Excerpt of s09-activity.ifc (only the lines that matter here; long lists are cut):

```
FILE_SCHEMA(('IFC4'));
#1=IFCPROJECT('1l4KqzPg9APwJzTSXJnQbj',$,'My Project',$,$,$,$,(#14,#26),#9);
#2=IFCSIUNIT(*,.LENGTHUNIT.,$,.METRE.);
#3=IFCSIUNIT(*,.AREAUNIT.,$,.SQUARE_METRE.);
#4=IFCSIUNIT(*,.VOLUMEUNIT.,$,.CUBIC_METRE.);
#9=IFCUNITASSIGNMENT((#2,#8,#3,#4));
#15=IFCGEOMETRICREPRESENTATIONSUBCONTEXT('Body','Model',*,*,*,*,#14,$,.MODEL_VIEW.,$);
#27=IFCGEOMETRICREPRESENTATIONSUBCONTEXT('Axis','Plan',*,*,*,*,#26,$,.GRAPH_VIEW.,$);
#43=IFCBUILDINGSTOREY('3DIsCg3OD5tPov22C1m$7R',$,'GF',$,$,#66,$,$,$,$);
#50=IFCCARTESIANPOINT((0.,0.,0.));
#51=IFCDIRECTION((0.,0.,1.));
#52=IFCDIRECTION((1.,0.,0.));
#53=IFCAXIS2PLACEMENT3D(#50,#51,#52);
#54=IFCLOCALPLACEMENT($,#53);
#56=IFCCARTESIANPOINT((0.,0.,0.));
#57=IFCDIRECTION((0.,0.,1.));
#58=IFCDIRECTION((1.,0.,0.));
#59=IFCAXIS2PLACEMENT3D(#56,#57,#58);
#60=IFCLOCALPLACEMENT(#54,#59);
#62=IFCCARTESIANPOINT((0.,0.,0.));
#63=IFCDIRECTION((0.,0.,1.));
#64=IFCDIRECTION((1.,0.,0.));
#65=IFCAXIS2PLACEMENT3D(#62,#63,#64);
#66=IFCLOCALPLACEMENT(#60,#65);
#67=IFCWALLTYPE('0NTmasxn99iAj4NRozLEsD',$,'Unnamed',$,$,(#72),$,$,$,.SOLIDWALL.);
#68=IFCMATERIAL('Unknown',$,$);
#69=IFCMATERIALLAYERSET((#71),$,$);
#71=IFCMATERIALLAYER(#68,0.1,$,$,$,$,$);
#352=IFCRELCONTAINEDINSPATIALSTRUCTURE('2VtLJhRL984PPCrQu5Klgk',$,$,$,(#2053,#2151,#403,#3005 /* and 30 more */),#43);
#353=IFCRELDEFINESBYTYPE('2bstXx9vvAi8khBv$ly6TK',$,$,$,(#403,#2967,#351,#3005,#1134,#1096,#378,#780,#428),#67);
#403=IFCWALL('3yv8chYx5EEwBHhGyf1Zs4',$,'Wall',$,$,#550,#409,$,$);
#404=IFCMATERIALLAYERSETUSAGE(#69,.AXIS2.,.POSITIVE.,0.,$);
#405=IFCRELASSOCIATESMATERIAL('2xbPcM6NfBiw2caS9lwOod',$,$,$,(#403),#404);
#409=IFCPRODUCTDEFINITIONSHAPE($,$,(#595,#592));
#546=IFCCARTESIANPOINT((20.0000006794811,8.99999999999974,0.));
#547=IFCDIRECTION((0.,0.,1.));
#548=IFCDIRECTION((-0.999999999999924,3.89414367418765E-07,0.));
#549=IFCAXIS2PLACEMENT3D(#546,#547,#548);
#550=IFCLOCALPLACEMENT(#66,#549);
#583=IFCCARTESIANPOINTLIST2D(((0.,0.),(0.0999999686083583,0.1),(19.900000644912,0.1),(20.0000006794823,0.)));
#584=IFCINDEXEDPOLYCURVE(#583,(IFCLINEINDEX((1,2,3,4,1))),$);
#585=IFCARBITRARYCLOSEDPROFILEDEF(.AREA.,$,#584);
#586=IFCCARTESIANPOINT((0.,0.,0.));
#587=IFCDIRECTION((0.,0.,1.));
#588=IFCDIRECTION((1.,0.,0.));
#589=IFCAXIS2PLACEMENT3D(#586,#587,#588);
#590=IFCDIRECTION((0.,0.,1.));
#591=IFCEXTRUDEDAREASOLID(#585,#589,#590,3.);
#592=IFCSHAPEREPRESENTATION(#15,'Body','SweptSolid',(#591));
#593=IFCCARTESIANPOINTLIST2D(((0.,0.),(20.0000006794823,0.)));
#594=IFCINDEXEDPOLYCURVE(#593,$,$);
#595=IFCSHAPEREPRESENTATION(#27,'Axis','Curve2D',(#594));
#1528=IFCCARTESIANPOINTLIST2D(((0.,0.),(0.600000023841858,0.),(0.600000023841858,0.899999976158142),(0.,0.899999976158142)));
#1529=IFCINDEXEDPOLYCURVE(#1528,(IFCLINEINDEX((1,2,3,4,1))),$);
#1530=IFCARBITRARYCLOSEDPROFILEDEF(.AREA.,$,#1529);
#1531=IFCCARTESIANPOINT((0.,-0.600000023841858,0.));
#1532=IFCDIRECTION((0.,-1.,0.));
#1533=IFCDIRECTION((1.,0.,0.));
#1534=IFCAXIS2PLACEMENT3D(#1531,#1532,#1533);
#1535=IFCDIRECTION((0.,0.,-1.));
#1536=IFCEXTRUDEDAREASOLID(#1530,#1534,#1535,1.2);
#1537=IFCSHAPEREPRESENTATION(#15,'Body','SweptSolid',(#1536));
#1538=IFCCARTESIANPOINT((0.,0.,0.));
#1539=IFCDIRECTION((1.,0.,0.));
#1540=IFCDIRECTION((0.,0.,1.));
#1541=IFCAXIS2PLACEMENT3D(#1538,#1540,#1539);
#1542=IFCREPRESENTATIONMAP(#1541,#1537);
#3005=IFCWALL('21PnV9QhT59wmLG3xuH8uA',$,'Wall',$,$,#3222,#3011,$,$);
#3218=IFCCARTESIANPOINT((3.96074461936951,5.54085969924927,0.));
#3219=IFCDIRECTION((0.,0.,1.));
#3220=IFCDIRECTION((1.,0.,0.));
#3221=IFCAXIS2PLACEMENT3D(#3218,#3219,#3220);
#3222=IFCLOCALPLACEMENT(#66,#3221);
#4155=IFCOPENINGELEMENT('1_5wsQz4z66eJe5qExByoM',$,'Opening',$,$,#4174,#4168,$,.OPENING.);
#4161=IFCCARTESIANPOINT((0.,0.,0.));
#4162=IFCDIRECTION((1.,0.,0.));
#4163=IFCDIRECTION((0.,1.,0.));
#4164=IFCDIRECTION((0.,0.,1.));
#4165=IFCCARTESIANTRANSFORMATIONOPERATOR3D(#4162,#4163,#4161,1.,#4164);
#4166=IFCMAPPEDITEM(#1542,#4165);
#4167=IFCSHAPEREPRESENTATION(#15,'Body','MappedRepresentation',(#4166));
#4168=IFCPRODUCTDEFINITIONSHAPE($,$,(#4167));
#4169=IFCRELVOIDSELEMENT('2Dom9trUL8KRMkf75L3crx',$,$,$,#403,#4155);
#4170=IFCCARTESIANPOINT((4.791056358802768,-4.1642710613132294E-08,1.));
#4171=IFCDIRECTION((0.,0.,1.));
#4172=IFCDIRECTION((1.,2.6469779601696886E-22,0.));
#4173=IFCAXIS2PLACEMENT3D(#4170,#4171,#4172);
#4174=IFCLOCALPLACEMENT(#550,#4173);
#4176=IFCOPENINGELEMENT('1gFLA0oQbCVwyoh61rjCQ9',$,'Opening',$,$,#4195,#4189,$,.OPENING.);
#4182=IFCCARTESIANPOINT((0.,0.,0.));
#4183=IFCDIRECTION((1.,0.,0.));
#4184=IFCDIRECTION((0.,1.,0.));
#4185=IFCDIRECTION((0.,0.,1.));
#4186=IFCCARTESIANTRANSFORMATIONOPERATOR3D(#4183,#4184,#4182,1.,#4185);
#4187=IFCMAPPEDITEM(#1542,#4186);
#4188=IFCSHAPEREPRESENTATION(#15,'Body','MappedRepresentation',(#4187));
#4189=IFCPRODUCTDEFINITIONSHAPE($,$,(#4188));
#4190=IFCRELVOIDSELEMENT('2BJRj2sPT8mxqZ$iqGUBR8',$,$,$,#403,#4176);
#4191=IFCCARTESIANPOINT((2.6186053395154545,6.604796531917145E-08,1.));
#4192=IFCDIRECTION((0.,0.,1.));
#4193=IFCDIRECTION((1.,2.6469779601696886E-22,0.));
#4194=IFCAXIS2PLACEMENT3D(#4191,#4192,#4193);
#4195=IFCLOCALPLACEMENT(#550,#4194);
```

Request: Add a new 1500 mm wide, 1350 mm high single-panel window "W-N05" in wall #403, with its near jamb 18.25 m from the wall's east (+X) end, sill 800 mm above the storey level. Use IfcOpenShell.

```python
import numpy as np
import ifcopenshell
import ifcopenshell.api.feature
import ifcopenshell.api.geometry
import ifcopenshell.api.root
import ifcopenshell.api.spatial
import ifcopenshell.geom
import ifcopenshell.util.element
import ifcopenshell.util.placement
import ifcopenshell.util.representation
import ifcopenshell.util.shape
import ifcopenshell.util.unit

model = ifcopenshell.open("s09-activity.ifc")
unit_scale = ifcopenshell.util.unit.calculate_unit_scale(model)
settings = ifcopenshell.geom.settings()


def volume(element):
    """Net volume in cubic metres, openings subtracted."""
    shape = ifcopenshell.geom.create_shape(settings, element)
    return ifcopenshell.util.shape.get_volume(shape.geometry)


wall = model.by_guid("3yv8chYx5EEwBHhGyf1Zs4")
storey = ifcopenshell.util.element.get_container(wall, ifc_class="IfcBuildingStorey")
context = ifcopenshell.util.representation.get_context(model, "Model", "Body", "MODEL_VIEW")
before = volume(wall)

width, height, from_end, sill = 1.5, 1.35, 18.25, 0.8  # metres

# The wall runs along its own X axis, and the end named is its -X end.
wall_shape = ifcopenshell.geom.create_shape(settings, wall)
x, y, z = ifcopenshell.util.shape.get_vertices(wall_shape.geometry).T
start = x.min() + from_end
face, thickness = float(y.min()), float(y.max() - y.min())
wall_matrix = ifcopenshell.util.placement.get_local_placement(wall.ObjectPlacement)
level = ifcopenshell.util.placement.get_local_placement(storey.ObjectPlacement)[2, 3]


def in_wall(x, y):
    """Placement at x, y metres in the wall's axes, at sill height."""
    matrix = wall_matrix.copy()
    matrix[:, 3] = wall_matrix @ np.array([x / unit_scale, y / unit_scale, 0.0, 1.0])
    matrix[2, 3] = level + sill / unit_scale
    return matrix


# Opening: a box that overshoots both wall faces by 50 mm.
opening = ifcopenshell.api.root.create_entity(model, ifc_class="IfcOpeningElement", predefined_type="OPENING")
box = ifcopenshell.api.geometry.add_wall_representation(
    model, context=context, length=width, height=height, thickness=thickness + 0.1
)
ifcopenshell.api.geometry.assign_representation(model, product=opening, representation=box)
ifcopenshell.api.geometry.edit_object_placement(model, product=opening, matrix=in_wall(start, face - 0.05), is_si=False)
ifcopenshell.api.feature.add_feature(model, feature=opening, element=wall)

window = ifcopenshell.api.root.create_entity(model, ifc_class="IfcWindow", name="W-N05", predefined_type="WINDOW")
window.OverallWidth, window.OverallHeight = width / unit_scale, height / unit_scale
window.PartitioningType = "SINGLE_PANEL"
body = ifcopenshell.api.geometry.add_window_representation(
    model,
    context=context,
    overall_width=window.OverallWidth,
    overall_height=window.OverallHeight,
    partition_type="SINGLE_PANEL",
)
ifcopenshell.api.geometry.assign_representation(model, product=window, representation=body)
ifcopenshell.api.spatial.assign_container(model, products=[window], relating_structure=storey)
ifcopenshell.api.feature.add_filling(model, opening=opening, element=window)

# Centre the window in the wall's thickness.
ifcopenshell.api.geometry.edit_object_placement(model, product=window, matrix=in_wall(start, face), is_si=False)
window_shape = ifcopenshell.geom.create_shape(settings, window)
depth = ifcopenshell.util.shape.get_vertices(window_shape.geometry)[:, 1]
offset = face + thickness / 2 - (depth.min() + depth.max()) / 2
ifcopenshell.api.geometry.edit_object_placement(model, product=window, matrix=in_wall(start, offset), is_si=False)

after = volume(wall)

print(f"wall volume {before:.3f} -> {after:.3f} m3")

model.write("s09-activity_rev.ifc")
```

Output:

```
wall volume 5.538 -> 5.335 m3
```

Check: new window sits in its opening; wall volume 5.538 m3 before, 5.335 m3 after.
